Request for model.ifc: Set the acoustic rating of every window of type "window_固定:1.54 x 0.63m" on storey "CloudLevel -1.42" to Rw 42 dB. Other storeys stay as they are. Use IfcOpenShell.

First a look at what the model holds.

```python
import ifcopenshell
import ifcopenshell.util.element

model = ifcopenshell.open("model.ifc")
print(model.schema)
storey = next(s for s in model.by_type("IfcBuildingStorey") if s.Name == "CloudLevel -1.42")
windows = [e for e in ifcopenshell.util.element.get_decomposition(storey) if e.is_a("IfcWindow")]
seen = {}
for e in windows:
    element_type = ifcopenshell.util.element.get_type(e)
    key = (element_type.Name if element_type != e and element_type else None, ifcopenshell.util.element.get_pset(e, "Pset_WindowCommon", "AcousticRating"))
    seen[key] = seen.get(key, 0) + 1
for (name, value), count in sorted(seen.items(), key=str):
    print(count, "x", name, "|", value)
```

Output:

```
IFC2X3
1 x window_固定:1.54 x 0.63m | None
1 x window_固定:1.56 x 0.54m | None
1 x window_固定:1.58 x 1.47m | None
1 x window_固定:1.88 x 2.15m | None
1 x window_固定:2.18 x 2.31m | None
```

```python
import ifcopenshell
import ifcopenshell.api.pset
import ifcopenshell.util.element

model = ifcopenshell.open("model.ifc")

storey = next(s for s in model.by_type("IfcBuildingStorey") if s.Name == "CloudLevel -1.42")
windows = [e for e in ifcopenshell.util.element.get_decomposition(storey) if e.is_a("IfcWindow")]

count = 0
for e in windows:
    element_type = ifcopenshell.util.element.get_type(e)
    if element_type in (None, e) or element_type.Name != "window_固定:1.54 x 0.63m":
        continue
    # add_pset returns the element's existing set when there is one.
    pset = ifcopenshell.api.pset.add_pset(model, product=e, name="Pset_WindowCommon")
    ifcopenshell.api.pset.edit_pset(model, pset=pset, properties={"AcousticRating": "Rw 42 dB"})
    count += 1

print(count, "windows updated")

model.write("model_v2.ifc")
```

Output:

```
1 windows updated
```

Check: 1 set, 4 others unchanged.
